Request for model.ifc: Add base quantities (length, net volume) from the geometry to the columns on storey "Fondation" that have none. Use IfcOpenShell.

First a look at what the model holds.

```python
import ifcopenshell
import ifcopenshell.util.element
import ifcopenshell.util.unit

model = ifcopenshell.open("model.ifc")
print(model.schema)
for unit_type in ("LENGTHUNIT", "AREAUNIT", "VOLUMEUNIT"):
    print(unit_type, ifcopenshell.util.unit.calculate_unit_scale(model, unit_type))
storey = next(s for s in model.by_type("IfcBuildingStorey") if s.Name == "Fondation")
columns = [e for e in ifcopenshell.util.element.get_decomposition(storey) if e.is_a("IfcColumn")]
for e in sorted(columns, key=lambda e: e.id()):
    print(e.id(), e.is_a(), e.Name, list(ifcopenshell.util.element.get_psets(e, qtos_only=True)), sep=" | ")
```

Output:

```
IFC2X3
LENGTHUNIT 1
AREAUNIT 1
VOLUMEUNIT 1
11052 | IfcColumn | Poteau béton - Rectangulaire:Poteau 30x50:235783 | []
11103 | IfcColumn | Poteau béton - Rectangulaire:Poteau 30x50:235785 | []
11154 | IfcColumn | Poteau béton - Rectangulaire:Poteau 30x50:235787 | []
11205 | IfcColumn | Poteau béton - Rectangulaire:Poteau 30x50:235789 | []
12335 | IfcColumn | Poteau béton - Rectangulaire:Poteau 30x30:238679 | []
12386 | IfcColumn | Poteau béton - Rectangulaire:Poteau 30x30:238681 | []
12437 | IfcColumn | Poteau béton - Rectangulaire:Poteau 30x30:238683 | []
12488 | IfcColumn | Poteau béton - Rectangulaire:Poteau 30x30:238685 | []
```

```python
import ifcopenshell
import ifcopenshell.api.pset
import ifcopenshell.geom
import ifcopenshell.util.element
import ifcopenshell.util.shape
import ifcopenshell.util.unit

model = ifcopenshell.open("model.ifc")
unit_scale = ifcopenshell.util.unit.calculate_unit_scale(model)
volume_scale = ifcopenshell.util.unit.calculate_unit_scale(model, "VOLUMEUNIT")
settings = ifcopenshell.geom.settings()

storey = next(s for s in model.by_type("IfcBuildingStorey") if s.Name == "Fondation")
columns = [e for e in ifcopenshell.util.element.get_decomposition(storey) if e.is_a("IfcColumn")]

for e in sorted(columns, key=lambda e: e.id()):
    if ifcopenshell.util.element.get_psets(e, qtos_only=True, should_inherit=False):
        continue
    # Geometry comes back in metres, in the element's own axes.
    shape = ifcopenshell.geom.create_shape(settings, e)
    values = {
        "Length": ifcopenshell.util.shape.get_z(shape.geometry) / unit_scale,
        "NetVolume": ifcopenshell.util.shape.get_volume(shape.geometry) / volume_scale,
    }
    qto = ifcopenshell.api.pset.add_qto(model, product=e, name="BaseQuantities")
    ifcopenshell.api.pset.edit_qto(model, qto=qto, properties=values)
    print(e.id(), {k: round(v, 3) for k, v in values.items()})

model.write("model-out.ifc")
```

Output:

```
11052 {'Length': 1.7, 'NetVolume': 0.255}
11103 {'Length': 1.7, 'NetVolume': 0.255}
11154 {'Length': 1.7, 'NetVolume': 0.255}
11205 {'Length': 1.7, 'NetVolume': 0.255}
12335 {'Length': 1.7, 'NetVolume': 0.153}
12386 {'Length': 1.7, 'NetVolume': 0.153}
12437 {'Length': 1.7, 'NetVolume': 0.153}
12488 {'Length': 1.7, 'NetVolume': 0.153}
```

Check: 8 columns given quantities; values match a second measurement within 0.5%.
